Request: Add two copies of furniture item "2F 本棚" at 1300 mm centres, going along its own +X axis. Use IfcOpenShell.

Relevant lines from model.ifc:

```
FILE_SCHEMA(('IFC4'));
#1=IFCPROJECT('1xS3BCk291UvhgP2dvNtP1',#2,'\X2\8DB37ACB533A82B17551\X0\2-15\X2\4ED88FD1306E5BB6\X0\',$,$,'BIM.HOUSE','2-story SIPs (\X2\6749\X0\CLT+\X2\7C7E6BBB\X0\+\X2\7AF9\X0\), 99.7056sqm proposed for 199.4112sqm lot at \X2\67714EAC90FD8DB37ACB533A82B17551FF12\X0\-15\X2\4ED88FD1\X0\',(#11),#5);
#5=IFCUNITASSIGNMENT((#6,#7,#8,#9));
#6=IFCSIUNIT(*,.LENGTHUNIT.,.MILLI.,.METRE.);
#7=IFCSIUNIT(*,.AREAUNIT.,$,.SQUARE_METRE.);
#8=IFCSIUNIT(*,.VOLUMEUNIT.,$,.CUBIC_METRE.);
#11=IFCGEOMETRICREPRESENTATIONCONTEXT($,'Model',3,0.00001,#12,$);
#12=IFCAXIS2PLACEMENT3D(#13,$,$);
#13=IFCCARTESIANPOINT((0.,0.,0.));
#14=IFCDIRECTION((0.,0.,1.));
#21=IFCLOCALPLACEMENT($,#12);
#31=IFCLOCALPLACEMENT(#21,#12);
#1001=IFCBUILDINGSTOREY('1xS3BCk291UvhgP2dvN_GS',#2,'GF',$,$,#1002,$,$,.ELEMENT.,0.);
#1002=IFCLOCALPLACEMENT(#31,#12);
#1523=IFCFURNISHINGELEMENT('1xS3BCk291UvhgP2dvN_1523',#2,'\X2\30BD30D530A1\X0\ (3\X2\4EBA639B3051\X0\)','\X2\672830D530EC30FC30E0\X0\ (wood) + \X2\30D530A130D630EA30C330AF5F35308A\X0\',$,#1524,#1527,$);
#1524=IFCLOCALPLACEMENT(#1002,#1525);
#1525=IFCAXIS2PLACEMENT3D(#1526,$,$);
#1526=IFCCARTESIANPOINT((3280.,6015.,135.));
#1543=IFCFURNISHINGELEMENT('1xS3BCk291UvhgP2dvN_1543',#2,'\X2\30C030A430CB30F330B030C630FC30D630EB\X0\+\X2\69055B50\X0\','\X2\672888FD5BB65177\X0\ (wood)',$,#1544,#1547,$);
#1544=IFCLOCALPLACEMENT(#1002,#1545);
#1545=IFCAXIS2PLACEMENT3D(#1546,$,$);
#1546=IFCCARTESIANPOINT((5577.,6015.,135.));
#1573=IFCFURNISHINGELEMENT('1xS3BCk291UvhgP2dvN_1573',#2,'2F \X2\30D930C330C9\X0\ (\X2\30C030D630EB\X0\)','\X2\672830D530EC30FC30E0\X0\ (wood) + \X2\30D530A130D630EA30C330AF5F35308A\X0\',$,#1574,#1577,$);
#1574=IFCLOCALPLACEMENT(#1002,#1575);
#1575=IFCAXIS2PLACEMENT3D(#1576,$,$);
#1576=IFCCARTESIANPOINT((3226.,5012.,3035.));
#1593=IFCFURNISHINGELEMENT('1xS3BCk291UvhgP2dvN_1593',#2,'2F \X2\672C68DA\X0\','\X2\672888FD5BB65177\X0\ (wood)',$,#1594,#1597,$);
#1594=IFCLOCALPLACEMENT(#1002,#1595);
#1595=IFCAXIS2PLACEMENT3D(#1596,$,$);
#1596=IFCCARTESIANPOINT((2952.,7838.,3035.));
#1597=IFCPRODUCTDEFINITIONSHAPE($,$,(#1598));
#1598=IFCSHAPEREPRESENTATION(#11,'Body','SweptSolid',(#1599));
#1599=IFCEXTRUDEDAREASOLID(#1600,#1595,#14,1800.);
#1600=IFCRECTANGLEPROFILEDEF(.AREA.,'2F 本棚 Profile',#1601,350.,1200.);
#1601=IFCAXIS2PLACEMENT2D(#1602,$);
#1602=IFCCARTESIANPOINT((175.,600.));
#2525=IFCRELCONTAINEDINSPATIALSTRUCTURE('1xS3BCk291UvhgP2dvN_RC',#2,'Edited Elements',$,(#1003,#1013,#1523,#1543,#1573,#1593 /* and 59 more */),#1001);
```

```python
import ifcopenshell
import ifcopenshell.api.geometry
import ifcopenshell.api.root
import ifcopenshell.util.element
import ifcopenshell.util.placement
import ifcopenshell.util.unit

model = ifcopenshell.open("model.ifc")
unit_scale = ifcopenshell.util.unit.calculate_unit_scale(model)


def reuse_history(source, copy):
    """copy_class also copies each property set's owner history, people and application; keep the originals."""
    for rel in copy.IsDefinedBy:
        if rel.is_a("IfcRelDefinesByProperties") and (history := rel.RelatingPropertyDefinition.OwnerHistory):
            rel.RelatingPropertyDefinition.OwnerHistory = source.OwnerHistory
            ifcopenshell.util.element.remove_deep2(model, history)


source = model.by_guid("1xS3BCk291UvhgP2dvN_1593")
base = ifcopenshell.util.placement.get_local_placement(source.ObjectPlacement)
step = base[:3, 0] * 1.3 / unit_scale

for i in range(1, 3):
    copy = ifcopenshell.api.root.copy_class(model, product=source)
    copy.Representation = ifcopenshell.util.element.copy_deep(
        model, source.Representation, exclude=["IfcGeometricRepresentationContext", "IfcRepresentationMap"]
    )
    reuse_history(source, copy)
    matrix = base.copy()
    matrix[:3, 3] += i * step
    print("added at", matrix[:3, 3].round(3) + 0.0)
    ifcopenshell.api.geometry.edit_object_placement(model, product=copy, matrix=matrix, is_si=False)

model.write("model_updated.ifc")
```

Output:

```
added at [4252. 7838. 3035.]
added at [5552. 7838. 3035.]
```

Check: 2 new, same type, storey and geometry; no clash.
